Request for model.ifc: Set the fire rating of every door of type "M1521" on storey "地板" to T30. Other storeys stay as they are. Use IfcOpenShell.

First a look at what the model holds.

```python
import ifcopenshell
import ifcopenshell.util.element

model = ifcopenshell.open("model.ifc")
print(model.schema)
storey = next(s for s in model.by_type("IfcBuildingStorey") if s.Name == "地板")
doors = [e for e in ifcopenshell.util.element.get_decomposition(storey) if e.is_a("IfcDoor")]
seen = {}
for e in doors:
    element_type = ifcopenshell.util.element.get_type(e)
    key = (element_type.Name if element_type != e and element_type else None, ifcopenshell.util.element.get_pset(e, "Pset_DoorCommon", "FireRating"))
    seen[key] = seen.get(key, 0) + 1
for (name, value), count in sorted(seen.items(), key=str):
    print(count, "x", name, "|", value)
```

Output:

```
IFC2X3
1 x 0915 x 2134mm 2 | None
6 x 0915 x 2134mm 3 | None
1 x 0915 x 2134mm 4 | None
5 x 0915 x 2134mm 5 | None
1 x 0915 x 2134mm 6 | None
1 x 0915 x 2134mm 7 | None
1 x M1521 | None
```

```python
import ifcopenshell
import ifcopenshell.api.pset
import ifcopenshell.util.element

model = ifcopenshell.open("model.ifc")

storey = next(s for s in model.by_type("IfcBuildingStorey") if s.Name == "地板")
doors = [e for e in ifcopenshell.util.element.get_decomposition(storey) if e.is_a("IfcDoor")]

count = 0
for e in doors:
    element_type = ifcopenshell.util.element.get_type(e)
    if element_type in (None, e) or element_type.Name != "M1521":
        continue
    # add_pset returns the element's existing set when there is one.
    pset = ifcopenshell.api.pset.add_pset(model, product=e, name="Pset_DoorCommon")
    ifcopenshell.api.pset.edit_pset(model, pset=pset, properties={"FireRating": "T30"})
    count += 1

print(count, "doors updated")

model.write("model_edited.ifc")
```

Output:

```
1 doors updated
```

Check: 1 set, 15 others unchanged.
